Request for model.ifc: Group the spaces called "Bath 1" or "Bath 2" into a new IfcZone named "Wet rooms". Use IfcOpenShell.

First a look at what the model holds.

```python
import ifcopenshell

model = ifcopenshell.open("model.ifc")
print(model.schema)
seen = {}
for space in model.by_type("IfcSpace"):
    seen[space.LongName] = seen.get(space.LongName, 0) + 1
for name, count in sorted(seen.items(), key=str):
    print(count, "x", name)
print("zones:", [z.Name for z in model.by_type("IfcZone")][:20])
```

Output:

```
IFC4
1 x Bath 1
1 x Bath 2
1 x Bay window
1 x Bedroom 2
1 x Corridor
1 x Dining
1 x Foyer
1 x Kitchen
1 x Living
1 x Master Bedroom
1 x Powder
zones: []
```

```python
import ifcopenshell
import ifcopenshell.api.group
import ifcopenshell.api.root

model = ifcopenshell.open("model.ifc")

names = {"Bath 1", "Bath 2"}
spaces = [s for s in model.by_type("IfcSpace") if s.LongName in names]

zone = ifcopenshell.api.root.create_entity(model, ifc_class="IfcZone", name="Wet rooms")
ifcopenshell.api.group.assign_group(model, products=spaces, group=zone)
print(len(spaces), "spaces in", zone.Name)

model.write("model_edited.ifc")
```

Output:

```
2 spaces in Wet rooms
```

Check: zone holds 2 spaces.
